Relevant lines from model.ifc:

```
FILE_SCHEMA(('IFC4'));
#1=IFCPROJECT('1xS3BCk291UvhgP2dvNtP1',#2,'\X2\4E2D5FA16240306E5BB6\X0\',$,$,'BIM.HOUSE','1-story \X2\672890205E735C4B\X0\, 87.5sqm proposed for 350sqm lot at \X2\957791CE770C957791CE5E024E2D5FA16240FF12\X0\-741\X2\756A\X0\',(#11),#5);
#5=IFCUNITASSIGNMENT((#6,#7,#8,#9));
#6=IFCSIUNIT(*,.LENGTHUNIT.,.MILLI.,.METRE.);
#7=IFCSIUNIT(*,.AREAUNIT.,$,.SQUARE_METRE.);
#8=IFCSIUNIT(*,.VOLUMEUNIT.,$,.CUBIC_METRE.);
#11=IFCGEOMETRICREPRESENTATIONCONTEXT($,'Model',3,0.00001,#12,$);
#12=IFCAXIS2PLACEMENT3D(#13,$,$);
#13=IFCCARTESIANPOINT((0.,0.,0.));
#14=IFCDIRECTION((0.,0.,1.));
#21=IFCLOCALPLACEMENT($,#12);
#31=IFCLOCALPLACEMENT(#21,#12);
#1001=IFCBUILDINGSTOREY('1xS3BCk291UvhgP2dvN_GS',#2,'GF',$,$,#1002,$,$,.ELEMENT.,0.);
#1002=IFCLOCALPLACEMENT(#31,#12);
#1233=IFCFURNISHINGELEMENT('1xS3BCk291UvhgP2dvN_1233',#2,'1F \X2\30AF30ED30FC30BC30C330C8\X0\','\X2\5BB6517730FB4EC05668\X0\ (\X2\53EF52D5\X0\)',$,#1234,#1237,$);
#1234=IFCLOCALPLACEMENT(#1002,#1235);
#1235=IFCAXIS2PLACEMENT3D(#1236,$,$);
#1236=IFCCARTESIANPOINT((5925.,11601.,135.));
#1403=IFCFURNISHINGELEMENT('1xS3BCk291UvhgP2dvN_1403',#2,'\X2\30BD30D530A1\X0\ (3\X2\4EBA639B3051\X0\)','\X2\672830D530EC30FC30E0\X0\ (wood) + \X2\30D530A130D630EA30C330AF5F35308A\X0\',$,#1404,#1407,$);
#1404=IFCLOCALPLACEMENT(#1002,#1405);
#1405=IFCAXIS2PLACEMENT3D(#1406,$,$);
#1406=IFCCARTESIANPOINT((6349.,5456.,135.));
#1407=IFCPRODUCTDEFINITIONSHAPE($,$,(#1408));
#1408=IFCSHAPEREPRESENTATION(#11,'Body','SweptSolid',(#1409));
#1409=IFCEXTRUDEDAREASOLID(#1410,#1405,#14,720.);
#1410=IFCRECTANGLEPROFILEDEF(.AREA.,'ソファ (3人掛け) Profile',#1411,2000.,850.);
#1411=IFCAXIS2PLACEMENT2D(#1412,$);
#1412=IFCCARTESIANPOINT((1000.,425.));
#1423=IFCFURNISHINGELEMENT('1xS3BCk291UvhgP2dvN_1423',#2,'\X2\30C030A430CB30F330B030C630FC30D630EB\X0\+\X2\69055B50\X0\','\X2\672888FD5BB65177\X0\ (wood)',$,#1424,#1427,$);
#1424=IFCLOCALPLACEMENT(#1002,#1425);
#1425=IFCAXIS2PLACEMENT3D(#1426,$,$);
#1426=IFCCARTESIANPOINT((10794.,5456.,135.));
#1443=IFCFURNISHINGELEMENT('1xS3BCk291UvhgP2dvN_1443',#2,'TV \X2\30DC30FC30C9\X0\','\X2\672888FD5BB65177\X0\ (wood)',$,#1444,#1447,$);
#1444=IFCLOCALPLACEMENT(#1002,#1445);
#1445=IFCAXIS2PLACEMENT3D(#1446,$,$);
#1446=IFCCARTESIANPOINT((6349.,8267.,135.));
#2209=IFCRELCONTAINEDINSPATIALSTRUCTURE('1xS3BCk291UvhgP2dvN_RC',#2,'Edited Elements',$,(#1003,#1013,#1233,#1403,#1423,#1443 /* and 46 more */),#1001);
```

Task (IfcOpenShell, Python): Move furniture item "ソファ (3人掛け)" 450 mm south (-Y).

```python
import ifcopenshell
import ifcopenshell.api.geometry
import ifcopenshell.util.placement
import ifcopenshell.util.unit

model = ifcopenshell.open("model.ifc")
unit_scale = ifcopenshell.util.unit.calculate_unit_scale(model)

item = model.by_guid("1xS3BCk291UvhgP2dvN_1403")
matrix = ifcopenshell.util.placement.get_local_placement(item.ObjectPlacement)
matrix[1, 3] -= 0.45 / unit_scale
ifcopenshell.api.geometry.edit_object_placement(model, product=item, matrix=matrix, is_si=False)

print(ifcopenshell.util.placement.get_local_placement(item.ObjectPlacement).round(3) + 0.0)

model.write("model-out.ifc")
```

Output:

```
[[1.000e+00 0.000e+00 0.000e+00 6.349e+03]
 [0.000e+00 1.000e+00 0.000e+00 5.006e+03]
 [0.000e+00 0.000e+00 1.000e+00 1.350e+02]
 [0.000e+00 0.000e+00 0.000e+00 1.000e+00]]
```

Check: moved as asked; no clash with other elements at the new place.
